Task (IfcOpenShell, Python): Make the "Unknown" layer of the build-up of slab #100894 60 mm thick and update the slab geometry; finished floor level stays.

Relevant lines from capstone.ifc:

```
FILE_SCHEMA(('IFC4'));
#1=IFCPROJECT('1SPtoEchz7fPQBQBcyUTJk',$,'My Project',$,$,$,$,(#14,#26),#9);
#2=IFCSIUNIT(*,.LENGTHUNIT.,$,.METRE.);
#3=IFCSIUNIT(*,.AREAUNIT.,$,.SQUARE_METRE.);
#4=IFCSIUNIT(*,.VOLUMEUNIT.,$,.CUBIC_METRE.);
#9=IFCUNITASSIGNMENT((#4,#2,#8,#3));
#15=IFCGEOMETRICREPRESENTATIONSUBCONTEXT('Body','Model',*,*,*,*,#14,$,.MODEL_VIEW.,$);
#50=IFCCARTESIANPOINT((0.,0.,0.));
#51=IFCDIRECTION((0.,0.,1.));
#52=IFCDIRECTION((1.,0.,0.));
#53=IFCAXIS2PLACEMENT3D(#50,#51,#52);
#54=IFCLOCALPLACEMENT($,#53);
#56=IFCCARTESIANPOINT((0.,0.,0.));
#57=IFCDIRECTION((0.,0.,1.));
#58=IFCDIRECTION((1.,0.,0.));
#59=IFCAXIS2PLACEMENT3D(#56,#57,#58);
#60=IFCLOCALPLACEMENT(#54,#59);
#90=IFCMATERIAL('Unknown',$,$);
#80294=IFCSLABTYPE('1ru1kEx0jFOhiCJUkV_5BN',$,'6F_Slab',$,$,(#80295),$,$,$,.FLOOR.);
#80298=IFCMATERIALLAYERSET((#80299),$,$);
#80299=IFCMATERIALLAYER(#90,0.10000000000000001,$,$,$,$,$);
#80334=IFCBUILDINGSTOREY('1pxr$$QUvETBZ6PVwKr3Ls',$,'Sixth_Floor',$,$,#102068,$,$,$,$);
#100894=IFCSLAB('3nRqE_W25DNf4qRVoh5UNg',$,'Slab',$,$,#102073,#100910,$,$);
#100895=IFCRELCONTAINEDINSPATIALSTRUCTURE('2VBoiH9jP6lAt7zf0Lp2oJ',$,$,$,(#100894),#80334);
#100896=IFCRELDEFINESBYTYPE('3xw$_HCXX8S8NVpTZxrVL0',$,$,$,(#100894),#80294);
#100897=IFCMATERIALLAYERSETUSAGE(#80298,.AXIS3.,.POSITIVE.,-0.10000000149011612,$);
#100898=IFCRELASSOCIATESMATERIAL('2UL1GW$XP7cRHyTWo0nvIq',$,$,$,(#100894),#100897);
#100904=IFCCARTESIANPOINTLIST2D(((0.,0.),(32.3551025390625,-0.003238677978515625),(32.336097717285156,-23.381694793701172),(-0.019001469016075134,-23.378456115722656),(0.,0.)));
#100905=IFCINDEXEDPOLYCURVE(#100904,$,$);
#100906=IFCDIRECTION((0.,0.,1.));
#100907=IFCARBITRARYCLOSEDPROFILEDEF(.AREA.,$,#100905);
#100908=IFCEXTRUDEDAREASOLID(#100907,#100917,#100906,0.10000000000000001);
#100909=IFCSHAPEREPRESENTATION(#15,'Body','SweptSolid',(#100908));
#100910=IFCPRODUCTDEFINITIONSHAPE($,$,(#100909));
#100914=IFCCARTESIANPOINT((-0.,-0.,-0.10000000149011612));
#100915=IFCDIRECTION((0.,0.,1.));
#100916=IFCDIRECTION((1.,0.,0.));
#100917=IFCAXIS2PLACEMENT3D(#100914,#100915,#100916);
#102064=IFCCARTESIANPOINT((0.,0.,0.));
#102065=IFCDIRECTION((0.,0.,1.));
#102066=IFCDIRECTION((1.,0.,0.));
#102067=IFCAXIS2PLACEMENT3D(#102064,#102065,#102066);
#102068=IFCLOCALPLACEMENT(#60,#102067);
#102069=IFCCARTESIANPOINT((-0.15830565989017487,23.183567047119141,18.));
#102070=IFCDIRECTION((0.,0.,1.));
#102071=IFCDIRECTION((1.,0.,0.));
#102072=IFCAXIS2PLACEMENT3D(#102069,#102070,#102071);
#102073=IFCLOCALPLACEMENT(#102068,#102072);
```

```python
import ifcopenshell
import ifcopenshell.util.element
import ifcopenshell.util.representation
import ifcopenshell.util.unit

model = ifcopenshell.open("capstone.ifc")
unit_scale = ifcopenshell.util.unit.calculate_unit_scale(model)

layer_set = model.by_id(80298)
layer = next(l for l in layer_set.MaterialLayers if l.Material and l.Material.Name == "Unknown")
change = 0.06 / unit_scale - layer.LayerThickness
layer.LayerThickness += change

# Geometry does not follow the layer set by itself.
slabs = [e for e in ifcopenshell.util.element.get_elements_by_material(model, layer_set) if e.is_a("IfcSlab")]
for slab in sorted(slabs, key=lambda e: e.id()):
    body = ifcopenshell.util.representation.get_representation(slab, "Model", "Body")
    solid = body.Items[0]
    old_depth = solid.Depth
    solid.Depth += change
    # Extruded upwards: lower the start of the extrusion so the top stays.
    x, y, z = solid.Position.Location.Coordinates
    solid.Position.Location = model.createIfcCartesianPoint((x, y, z - change))
    print(slab.id(), f"{old_depth:g} -> {solid.Depth:g}")

# The layers are counted up from the underside, which has moved.
for usage in {ifcopenshell.util.element.get_material(slab) for slab in slabs}:
    usage.OffsetFromReferenceLine -= change

model.write("capstone_edited.ifc")
```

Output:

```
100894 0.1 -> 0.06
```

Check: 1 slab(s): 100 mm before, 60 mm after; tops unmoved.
